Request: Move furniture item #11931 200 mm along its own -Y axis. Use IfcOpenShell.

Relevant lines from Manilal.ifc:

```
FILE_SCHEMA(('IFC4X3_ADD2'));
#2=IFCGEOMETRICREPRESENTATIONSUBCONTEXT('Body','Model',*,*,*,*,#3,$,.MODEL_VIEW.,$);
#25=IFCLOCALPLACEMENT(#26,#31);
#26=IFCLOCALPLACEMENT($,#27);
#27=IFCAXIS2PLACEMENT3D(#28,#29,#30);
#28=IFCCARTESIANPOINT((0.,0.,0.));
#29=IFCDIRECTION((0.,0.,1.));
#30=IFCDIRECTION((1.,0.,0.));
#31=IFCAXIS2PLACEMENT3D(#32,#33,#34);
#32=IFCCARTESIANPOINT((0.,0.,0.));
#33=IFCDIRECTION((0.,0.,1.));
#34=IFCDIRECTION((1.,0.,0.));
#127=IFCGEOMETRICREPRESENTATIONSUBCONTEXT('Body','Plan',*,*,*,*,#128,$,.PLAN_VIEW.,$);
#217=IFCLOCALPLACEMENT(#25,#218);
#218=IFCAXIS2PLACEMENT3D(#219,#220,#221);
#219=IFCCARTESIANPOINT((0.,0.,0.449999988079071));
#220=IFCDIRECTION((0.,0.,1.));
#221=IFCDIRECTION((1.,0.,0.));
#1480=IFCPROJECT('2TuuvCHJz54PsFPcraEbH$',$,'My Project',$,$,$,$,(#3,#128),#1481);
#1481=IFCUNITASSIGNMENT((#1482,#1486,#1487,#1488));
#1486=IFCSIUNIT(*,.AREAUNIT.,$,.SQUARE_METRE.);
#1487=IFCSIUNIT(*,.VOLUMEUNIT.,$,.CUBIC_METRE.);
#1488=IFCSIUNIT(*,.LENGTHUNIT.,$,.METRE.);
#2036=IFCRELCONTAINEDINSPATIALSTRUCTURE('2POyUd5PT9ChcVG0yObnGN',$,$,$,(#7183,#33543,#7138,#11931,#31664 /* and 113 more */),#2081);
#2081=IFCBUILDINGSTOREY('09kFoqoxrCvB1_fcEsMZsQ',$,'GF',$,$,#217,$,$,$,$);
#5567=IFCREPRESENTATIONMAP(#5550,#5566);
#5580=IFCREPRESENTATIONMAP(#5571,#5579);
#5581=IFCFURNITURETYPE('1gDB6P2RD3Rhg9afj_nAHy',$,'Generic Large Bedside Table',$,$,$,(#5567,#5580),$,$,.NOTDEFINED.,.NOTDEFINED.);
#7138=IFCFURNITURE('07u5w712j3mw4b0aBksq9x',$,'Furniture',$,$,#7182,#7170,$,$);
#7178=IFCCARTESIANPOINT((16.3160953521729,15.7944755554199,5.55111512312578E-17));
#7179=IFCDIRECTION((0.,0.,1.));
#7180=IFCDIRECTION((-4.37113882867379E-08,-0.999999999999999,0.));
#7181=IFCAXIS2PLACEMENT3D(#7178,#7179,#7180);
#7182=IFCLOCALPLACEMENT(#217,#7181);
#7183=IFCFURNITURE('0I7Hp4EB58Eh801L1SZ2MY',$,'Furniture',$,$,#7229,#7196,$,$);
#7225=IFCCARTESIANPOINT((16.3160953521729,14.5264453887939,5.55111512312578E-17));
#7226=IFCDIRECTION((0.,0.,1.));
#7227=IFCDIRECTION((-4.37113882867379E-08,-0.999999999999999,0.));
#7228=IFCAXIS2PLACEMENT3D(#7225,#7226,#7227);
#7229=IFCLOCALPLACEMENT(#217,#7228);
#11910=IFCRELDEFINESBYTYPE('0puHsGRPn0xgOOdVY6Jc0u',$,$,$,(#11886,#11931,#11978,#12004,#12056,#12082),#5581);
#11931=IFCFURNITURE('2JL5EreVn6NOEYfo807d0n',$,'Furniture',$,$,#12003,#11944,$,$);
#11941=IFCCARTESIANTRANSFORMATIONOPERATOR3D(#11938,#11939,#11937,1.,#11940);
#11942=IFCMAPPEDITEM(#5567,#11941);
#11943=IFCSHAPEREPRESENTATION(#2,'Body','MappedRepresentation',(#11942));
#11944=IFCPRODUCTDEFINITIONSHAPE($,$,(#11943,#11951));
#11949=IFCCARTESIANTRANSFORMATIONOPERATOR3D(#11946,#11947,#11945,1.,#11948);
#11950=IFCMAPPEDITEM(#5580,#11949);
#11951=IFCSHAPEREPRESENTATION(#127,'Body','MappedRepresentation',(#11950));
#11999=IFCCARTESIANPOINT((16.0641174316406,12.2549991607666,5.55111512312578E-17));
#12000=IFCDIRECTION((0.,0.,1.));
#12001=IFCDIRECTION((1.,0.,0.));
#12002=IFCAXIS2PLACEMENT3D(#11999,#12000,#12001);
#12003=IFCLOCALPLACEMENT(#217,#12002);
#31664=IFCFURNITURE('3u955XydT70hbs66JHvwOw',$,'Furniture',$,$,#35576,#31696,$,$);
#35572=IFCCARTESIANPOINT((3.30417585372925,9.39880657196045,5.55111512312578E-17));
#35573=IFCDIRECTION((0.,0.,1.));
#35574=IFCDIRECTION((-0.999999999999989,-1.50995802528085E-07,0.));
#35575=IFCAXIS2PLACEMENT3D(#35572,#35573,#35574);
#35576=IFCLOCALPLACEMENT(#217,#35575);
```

```python
import ifcopenshell
import ifcopenshell.api.geometry
import ifcopenshell.util.placement
import ifcopenshell.util.unit

model = ifcopenshell.open("Manilal.ifc")
unit_scale = ifcopenshell.util.unit.calculate_unit_scale(model)

item = model.by_guid("2JL5EreVn6NOEYfo807d0n")
matrix = ifcopenshell.util.placement.get_local_placement(item.ObjectPlacement)
matrix[:3, 3] -= matrix[:3, 1] * 0.2 / unit_scale
ifcopenshell.api.geometry.edit_object_placement(model, product=item, matrix=matrix, is_si=False)

print(ifcopenshell.util.placement.get_local_placement(item.ObjectPlacement).round(3) + 0.0)

model.write("Manilal-out.ifc")
```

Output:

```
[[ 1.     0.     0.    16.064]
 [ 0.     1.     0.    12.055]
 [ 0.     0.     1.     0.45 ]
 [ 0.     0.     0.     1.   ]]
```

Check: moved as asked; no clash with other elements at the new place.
